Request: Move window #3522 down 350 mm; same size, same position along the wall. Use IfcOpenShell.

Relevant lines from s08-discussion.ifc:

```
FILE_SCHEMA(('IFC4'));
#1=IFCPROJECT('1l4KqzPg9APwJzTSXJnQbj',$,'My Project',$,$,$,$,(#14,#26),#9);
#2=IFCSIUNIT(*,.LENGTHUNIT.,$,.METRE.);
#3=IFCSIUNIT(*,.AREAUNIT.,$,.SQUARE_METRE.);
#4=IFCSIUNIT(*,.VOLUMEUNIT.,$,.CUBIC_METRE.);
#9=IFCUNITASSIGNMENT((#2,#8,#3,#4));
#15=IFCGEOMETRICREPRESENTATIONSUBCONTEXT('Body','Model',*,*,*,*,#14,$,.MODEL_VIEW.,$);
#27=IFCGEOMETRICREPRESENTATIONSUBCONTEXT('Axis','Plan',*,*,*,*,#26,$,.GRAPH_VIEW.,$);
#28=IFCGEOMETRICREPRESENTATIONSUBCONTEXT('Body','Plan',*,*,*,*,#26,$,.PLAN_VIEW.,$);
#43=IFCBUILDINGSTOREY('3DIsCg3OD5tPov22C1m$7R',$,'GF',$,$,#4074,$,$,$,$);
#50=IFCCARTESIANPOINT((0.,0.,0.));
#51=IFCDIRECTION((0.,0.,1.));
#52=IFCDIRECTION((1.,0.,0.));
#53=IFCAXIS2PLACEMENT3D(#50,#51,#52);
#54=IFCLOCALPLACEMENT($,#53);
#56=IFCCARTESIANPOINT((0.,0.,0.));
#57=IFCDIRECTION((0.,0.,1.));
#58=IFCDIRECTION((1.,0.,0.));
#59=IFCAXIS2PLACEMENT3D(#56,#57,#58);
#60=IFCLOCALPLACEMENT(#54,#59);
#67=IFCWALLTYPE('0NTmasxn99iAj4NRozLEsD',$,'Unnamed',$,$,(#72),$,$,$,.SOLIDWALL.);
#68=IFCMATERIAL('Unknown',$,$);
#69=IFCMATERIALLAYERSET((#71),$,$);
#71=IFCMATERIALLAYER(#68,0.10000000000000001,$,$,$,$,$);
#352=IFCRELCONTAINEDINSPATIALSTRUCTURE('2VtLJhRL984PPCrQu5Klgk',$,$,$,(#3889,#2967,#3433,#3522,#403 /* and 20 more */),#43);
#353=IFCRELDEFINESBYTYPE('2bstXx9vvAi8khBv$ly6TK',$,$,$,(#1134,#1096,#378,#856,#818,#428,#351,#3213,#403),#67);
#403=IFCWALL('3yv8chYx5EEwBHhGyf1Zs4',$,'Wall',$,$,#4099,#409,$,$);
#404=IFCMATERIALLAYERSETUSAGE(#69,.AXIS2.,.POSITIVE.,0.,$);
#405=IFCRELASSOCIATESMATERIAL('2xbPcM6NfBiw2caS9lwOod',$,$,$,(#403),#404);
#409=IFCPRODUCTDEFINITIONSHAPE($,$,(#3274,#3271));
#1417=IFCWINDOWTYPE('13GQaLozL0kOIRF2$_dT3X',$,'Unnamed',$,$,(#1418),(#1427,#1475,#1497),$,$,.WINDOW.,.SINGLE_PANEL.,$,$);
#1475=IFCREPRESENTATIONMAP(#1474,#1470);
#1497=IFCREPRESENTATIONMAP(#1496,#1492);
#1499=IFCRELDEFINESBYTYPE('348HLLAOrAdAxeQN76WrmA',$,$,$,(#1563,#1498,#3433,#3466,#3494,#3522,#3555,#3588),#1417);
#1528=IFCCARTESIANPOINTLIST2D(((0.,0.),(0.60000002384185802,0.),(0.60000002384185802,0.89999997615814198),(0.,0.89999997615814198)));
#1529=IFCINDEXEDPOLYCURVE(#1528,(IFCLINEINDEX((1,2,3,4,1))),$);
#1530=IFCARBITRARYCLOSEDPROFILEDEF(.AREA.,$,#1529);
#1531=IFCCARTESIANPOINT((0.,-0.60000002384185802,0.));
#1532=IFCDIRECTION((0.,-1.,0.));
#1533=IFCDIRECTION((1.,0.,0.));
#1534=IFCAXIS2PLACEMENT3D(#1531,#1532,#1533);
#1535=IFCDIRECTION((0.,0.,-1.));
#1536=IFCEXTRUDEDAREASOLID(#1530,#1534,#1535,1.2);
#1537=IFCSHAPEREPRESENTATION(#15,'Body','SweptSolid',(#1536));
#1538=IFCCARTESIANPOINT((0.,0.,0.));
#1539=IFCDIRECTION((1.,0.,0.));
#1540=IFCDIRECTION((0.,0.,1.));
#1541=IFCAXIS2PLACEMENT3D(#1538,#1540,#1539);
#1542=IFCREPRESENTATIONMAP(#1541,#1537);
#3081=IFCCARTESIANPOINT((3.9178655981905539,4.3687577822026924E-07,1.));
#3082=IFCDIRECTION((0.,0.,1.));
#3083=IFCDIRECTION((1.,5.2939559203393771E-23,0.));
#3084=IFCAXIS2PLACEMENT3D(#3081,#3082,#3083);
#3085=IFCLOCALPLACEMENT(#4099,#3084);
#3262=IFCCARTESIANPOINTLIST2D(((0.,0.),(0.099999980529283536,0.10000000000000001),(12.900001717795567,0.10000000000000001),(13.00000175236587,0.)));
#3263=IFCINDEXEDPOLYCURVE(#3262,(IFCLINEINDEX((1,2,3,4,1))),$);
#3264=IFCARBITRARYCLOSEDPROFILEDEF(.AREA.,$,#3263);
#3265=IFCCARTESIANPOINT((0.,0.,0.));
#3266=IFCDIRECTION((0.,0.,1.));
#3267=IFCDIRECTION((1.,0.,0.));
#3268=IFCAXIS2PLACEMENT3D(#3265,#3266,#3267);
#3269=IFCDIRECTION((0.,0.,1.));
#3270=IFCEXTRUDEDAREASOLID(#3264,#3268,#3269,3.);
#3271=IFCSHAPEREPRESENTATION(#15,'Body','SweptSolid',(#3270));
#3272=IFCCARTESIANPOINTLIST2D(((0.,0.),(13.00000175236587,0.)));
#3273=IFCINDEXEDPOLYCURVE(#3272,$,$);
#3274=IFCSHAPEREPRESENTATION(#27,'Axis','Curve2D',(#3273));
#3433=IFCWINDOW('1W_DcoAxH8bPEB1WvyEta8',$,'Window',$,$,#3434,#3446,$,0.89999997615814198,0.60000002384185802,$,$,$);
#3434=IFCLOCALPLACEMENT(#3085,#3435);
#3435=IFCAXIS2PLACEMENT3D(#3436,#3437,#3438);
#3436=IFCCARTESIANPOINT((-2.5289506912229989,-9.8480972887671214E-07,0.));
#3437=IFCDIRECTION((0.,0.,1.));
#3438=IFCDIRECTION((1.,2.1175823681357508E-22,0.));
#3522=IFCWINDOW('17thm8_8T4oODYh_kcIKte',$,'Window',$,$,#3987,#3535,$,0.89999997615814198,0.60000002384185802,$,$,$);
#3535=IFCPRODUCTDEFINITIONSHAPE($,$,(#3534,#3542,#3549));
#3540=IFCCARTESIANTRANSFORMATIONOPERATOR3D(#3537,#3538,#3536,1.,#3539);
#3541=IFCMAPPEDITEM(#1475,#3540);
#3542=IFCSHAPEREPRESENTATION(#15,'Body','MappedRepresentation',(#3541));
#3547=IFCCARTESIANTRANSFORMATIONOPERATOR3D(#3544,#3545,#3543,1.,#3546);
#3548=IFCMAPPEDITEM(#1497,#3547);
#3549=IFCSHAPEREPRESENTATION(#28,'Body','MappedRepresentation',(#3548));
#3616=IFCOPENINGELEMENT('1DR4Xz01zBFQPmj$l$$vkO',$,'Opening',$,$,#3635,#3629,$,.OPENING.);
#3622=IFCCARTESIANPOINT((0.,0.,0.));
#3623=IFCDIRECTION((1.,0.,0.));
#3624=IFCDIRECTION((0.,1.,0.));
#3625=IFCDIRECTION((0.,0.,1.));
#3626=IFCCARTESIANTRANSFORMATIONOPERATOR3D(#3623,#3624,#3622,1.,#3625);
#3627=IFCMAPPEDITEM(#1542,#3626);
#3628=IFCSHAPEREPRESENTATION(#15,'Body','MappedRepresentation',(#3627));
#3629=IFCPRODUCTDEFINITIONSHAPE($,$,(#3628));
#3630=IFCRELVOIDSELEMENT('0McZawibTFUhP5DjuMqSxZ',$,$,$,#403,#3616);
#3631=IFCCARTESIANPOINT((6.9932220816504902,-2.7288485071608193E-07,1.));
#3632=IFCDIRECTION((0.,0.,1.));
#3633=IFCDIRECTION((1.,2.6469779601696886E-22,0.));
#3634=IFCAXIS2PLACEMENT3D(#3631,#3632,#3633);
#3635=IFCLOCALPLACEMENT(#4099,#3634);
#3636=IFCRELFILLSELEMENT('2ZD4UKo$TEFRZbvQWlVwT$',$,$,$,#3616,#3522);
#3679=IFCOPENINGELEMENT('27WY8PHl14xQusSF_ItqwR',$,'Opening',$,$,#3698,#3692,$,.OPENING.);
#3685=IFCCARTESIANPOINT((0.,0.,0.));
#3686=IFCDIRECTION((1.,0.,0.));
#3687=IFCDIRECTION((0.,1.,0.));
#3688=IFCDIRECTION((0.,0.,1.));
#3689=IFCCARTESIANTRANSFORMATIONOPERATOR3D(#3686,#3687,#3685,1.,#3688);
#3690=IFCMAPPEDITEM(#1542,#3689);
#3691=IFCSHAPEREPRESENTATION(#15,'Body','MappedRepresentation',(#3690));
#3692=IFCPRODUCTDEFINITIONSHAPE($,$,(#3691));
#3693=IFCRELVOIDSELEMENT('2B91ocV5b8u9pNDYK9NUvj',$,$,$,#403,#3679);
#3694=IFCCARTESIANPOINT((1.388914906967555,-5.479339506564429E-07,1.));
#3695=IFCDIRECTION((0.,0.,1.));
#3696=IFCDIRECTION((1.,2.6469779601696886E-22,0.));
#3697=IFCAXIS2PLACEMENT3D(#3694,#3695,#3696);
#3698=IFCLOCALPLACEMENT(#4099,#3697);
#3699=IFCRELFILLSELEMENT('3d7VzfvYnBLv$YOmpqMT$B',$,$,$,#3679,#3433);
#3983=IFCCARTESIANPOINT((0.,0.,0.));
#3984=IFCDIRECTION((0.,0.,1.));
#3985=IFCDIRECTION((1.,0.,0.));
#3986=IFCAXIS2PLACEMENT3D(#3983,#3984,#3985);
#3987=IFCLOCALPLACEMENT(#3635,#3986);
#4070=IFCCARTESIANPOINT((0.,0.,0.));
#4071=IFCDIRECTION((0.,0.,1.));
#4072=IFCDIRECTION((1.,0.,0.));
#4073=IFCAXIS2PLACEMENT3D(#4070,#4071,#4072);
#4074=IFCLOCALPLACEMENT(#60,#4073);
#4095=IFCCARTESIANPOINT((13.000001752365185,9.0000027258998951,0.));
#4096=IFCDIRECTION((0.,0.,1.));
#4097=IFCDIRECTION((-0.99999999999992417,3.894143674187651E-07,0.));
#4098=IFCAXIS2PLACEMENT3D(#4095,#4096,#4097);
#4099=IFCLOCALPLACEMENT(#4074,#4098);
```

```python
import numpy as np
import ifcopenshell
import ifcopenshell.api.geometry
import ifcopenshell.util.placement
import ifcopenshell.util.unit

model = ifcopenshell.open("s08-discussion.ifc")
unit_scale = ifcopenshell.util.unit.calculate_unit_scale(model)

window = model.by_guid("17thm8_8T4oODYh_kcIKte")
opening = window.FillsVoids[0].RelatingOpeningElement
dz = -0.35 / unit_scale

shift = np.array([0.0, 0.0, dz])
# The window is placed relative to its opening, so it follows when the opening moves.
matrix = ifcopenshell.util.placement.get_local_placement(opening.ObjectPlacement)
matrix[:3, 3] += shift
ifcopenshell.api.geometry.edit_object_placement(
    model, product=opening, matrix=matrix, is_si=False, should_transform_children=True
)

print(f"moved by {dz * unit_scale:+.3f} m")

model.write("s08-discussion-out.ifc")
```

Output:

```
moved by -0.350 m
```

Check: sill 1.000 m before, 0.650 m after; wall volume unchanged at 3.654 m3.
